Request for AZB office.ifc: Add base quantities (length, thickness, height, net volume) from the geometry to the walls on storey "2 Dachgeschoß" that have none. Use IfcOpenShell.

First a look at what the model holds.

```python
import ifcopenshell
import ifcopenshell.util.element
import ifcopenshell.util.unit

model = ifcopenshell.open("AZB office.ifc")
print(model.schema)
for unit_type in ("LENGTHUNIT", "AREAUNIT", "VOLUMEUNIT"):
    print(unit_type, ifcopenshell.util.unit.calculate_unit_scale(model, unit_type))
storey = next(s for s in model.by_type("IfcBuildingStorey") if s.Name == "2 Dachgeschoß")
walls = [e for e in ifcopenshell.util.element.get_decomposition(storey) if e.is_a("IfcWall")]
for e in sorted(walls, key=lambda e: e.id()):
    print(e.id(), e.is_a(), e.Name, list(ifcopenshell.util.element.get_psets(e, qtos_only=True)), sep=" | ")
```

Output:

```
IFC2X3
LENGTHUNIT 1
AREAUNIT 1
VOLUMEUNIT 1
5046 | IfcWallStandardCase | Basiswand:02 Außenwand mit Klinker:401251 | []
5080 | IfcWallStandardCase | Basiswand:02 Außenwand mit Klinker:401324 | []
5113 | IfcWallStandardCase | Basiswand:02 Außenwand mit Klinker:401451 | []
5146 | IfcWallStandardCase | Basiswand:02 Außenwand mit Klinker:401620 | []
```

```python
import ifcopenshell
import ifcopenshell.api.pset
import ifcopenshell.geom
import ifcopenshell.util.element
import ifcopenshell.util.shape
import ifcopenshell.util.unit

model = ifcopenshell.open("AZB office.ifc")
unit_scale = ifcopenshell.util.unit.calculate_unit_scale(model)
volume_scale = ifcopenshell.util.unit.calculate_unit_scale(model, "VOLUMEUNIT")
settings = ifcopenshell.geom.settings()

storey = next(s for s in model.by_type("IfcBuildingStorey") if s.Name == "2 Dachgeschoß")
walls = [e for e in ifcopenshell.util.element.get_decomposition(storey) if e.is_a("IfcWall")]

for e in sorted(walls, key=lambda e: e.id()):
    if ifcopenshell.util.element.get_psets(e, qtos_only=True, should_inherit=False):
        continue
    # Geometry comes back in metres, in the element's own axes.
    shape = ifcopenshell.geom.create_shape(settings, e)
    values = {
        "Length": ifcopenshell.util.shape.get_x(shape.geometry) / unit_scale,
        "Width": ifcopenshell.util.shape.get_y(shape.geometry) / unit_scale,
        "Height": ifcopenshell.util.shape.get_z(shape.geometry) / unit_scale,
        "NetVolume": ifcopenshell.util.shape.get_volume(shape.geometry) / volume_scale,
    }
    qto = ifcopenshell.api.pset.add_qto(model, product=e, name="BaseQuantities")
    ifcopenshell.api.pset.edit_qto(model, qto=qto, properties=values)
    print(e.id(), {k: round(v, 3) for k, v in values.items()})

model.write("AZB office_rev.ifc")
```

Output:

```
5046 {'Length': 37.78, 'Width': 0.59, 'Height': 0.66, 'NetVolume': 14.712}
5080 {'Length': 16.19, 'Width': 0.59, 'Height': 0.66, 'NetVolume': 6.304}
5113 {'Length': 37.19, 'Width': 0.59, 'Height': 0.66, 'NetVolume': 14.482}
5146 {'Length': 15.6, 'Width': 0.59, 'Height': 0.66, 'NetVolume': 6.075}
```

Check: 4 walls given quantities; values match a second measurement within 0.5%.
